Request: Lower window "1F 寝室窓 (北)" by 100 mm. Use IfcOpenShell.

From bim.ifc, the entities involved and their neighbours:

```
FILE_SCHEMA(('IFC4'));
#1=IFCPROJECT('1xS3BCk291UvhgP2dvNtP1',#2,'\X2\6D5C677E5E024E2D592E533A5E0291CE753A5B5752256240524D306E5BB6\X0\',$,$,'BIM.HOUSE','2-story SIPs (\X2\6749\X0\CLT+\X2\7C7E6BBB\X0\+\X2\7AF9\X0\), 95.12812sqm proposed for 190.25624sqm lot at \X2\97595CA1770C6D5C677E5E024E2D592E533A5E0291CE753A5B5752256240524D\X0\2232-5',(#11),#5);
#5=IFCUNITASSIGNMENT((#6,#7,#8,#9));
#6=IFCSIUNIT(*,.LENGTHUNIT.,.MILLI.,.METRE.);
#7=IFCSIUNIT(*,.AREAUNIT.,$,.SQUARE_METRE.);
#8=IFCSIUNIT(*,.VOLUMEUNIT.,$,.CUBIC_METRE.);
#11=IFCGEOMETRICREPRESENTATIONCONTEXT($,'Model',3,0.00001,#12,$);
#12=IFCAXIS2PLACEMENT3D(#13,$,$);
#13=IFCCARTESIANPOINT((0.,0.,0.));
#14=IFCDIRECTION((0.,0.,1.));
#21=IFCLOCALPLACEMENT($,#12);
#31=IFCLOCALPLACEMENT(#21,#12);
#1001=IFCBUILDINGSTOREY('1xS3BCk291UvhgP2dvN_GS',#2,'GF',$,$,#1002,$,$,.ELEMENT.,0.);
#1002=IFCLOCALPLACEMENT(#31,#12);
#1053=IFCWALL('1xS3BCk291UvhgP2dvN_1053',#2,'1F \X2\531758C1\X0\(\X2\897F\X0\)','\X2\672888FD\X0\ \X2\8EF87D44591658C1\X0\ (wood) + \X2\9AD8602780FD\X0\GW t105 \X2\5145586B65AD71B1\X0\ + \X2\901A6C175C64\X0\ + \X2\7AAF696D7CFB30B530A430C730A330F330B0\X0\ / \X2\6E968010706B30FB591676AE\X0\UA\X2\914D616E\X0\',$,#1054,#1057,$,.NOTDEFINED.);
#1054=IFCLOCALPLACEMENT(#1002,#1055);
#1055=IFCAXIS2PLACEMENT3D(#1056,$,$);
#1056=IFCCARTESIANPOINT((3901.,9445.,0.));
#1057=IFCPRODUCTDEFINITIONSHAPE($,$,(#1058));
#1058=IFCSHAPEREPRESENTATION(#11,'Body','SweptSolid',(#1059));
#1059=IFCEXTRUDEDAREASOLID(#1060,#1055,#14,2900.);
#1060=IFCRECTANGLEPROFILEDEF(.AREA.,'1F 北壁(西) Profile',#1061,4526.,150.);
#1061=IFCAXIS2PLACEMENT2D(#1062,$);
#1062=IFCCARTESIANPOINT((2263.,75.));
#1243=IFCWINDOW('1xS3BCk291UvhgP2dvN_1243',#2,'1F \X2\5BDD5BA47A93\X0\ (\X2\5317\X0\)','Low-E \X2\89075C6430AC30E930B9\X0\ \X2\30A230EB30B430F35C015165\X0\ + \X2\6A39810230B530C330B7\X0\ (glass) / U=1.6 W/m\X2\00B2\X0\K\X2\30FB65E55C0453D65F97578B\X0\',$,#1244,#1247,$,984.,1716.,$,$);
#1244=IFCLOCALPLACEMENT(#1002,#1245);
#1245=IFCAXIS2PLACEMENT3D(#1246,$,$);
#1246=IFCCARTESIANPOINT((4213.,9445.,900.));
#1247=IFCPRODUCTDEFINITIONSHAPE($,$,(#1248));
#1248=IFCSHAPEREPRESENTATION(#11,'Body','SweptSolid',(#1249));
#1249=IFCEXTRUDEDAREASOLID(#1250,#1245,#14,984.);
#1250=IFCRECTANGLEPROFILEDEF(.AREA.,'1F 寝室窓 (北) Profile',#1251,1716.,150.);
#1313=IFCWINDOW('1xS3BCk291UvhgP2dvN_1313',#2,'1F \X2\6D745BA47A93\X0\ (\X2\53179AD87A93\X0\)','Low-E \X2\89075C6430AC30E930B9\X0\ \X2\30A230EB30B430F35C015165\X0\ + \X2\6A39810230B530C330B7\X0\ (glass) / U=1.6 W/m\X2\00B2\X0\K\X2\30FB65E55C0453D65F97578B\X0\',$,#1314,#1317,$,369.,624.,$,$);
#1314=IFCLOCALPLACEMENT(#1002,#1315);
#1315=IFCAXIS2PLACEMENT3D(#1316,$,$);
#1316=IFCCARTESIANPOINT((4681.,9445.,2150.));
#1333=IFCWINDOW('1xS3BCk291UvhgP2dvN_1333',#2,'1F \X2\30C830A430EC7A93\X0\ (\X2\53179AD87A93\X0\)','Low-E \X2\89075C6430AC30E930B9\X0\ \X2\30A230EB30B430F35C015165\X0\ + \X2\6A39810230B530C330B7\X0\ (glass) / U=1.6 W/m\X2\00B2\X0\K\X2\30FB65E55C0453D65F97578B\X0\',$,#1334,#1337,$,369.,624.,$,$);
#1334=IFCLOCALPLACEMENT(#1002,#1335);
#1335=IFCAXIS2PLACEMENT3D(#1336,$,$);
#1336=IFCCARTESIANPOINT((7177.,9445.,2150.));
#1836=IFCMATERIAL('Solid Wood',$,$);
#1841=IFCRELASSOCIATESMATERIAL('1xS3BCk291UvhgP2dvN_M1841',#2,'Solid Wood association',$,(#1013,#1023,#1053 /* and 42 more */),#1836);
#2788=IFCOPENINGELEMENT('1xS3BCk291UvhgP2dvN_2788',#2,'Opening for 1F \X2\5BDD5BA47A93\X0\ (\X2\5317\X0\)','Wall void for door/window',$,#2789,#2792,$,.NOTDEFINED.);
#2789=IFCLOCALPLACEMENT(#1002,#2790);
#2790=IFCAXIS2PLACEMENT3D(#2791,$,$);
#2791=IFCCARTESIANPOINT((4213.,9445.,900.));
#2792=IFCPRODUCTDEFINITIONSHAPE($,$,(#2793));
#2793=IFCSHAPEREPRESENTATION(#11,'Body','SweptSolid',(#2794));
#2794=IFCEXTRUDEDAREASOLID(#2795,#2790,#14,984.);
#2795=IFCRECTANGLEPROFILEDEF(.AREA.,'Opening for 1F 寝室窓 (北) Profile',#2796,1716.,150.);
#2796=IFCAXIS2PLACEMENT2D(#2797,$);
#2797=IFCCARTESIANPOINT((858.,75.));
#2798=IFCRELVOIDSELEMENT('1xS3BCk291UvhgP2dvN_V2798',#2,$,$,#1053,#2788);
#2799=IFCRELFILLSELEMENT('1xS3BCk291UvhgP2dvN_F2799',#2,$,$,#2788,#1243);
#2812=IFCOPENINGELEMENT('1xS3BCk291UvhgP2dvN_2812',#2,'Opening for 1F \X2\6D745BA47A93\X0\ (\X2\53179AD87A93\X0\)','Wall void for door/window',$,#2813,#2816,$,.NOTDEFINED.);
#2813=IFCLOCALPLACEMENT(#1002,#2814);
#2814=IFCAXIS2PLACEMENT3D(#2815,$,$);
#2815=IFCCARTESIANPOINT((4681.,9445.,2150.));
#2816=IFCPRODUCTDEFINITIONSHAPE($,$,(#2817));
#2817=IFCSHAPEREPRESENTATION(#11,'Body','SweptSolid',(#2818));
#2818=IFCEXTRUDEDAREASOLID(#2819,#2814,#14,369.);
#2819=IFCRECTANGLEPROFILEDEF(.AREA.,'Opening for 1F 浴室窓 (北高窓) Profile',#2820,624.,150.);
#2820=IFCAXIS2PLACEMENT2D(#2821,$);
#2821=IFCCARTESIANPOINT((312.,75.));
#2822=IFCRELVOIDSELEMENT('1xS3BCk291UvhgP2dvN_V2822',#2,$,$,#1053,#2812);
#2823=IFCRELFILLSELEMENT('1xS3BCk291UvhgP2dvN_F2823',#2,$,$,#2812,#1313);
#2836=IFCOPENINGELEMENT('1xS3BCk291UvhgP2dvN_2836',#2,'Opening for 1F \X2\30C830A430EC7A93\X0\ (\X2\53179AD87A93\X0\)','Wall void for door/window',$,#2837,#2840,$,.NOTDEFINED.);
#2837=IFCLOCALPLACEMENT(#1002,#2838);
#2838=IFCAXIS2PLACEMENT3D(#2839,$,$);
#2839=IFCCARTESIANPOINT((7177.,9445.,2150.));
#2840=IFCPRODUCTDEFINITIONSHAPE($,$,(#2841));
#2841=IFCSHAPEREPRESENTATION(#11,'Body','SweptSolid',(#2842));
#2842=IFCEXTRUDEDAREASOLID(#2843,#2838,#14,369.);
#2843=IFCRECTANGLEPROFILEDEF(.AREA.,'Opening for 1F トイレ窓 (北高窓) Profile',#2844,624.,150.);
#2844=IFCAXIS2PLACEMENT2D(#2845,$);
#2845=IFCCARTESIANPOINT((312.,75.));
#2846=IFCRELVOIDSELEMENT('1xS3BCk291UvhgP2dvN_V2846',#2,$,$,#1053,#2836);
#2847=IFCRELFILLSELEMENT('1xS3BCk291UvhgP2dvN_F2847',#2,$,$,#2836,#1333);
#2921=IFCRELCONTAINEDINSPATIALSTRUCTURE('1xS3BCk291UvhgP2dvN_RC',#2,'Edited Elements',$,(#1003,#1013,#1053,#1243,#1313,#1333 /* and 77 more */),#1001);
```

```python
import numpy as np
import ifcopenshell
import ifcopenshell.api.geometry
import ifcopenshell.util.placement
import ifcopenshell.util.unit

model = ifcopenshell.open("bim.ifc")
unit_scale = ifcopenshell.util.unit.calculate_unit_scale(model)

window = model.by_guid("1xS3BCk291UvhgP2dvN_1243")
opening = window.FillsVoids[0].RelatingOpeningElement
dz = -0.1 / unit_scale

shift = np.array([0.0, 0.0, dz])
# The window is not placed relative to its opening, so move both.
for product in (opening, window):
    matrix = ifcopenshell.util.placement.get_local_placement(product.ObjectPlacement)
    matrix[:3, 3] += shift
    ifcopenshell.api.geometry.edit_object_placement(model, product=product, matrix=matrix, is_si=False)

print(f"moved by {dz * unit_scale:+.3f} m")

model.write("bim_rev.ifc")
```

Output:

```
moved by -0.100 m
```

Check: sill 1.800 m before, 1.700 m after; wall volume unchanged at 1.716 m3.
